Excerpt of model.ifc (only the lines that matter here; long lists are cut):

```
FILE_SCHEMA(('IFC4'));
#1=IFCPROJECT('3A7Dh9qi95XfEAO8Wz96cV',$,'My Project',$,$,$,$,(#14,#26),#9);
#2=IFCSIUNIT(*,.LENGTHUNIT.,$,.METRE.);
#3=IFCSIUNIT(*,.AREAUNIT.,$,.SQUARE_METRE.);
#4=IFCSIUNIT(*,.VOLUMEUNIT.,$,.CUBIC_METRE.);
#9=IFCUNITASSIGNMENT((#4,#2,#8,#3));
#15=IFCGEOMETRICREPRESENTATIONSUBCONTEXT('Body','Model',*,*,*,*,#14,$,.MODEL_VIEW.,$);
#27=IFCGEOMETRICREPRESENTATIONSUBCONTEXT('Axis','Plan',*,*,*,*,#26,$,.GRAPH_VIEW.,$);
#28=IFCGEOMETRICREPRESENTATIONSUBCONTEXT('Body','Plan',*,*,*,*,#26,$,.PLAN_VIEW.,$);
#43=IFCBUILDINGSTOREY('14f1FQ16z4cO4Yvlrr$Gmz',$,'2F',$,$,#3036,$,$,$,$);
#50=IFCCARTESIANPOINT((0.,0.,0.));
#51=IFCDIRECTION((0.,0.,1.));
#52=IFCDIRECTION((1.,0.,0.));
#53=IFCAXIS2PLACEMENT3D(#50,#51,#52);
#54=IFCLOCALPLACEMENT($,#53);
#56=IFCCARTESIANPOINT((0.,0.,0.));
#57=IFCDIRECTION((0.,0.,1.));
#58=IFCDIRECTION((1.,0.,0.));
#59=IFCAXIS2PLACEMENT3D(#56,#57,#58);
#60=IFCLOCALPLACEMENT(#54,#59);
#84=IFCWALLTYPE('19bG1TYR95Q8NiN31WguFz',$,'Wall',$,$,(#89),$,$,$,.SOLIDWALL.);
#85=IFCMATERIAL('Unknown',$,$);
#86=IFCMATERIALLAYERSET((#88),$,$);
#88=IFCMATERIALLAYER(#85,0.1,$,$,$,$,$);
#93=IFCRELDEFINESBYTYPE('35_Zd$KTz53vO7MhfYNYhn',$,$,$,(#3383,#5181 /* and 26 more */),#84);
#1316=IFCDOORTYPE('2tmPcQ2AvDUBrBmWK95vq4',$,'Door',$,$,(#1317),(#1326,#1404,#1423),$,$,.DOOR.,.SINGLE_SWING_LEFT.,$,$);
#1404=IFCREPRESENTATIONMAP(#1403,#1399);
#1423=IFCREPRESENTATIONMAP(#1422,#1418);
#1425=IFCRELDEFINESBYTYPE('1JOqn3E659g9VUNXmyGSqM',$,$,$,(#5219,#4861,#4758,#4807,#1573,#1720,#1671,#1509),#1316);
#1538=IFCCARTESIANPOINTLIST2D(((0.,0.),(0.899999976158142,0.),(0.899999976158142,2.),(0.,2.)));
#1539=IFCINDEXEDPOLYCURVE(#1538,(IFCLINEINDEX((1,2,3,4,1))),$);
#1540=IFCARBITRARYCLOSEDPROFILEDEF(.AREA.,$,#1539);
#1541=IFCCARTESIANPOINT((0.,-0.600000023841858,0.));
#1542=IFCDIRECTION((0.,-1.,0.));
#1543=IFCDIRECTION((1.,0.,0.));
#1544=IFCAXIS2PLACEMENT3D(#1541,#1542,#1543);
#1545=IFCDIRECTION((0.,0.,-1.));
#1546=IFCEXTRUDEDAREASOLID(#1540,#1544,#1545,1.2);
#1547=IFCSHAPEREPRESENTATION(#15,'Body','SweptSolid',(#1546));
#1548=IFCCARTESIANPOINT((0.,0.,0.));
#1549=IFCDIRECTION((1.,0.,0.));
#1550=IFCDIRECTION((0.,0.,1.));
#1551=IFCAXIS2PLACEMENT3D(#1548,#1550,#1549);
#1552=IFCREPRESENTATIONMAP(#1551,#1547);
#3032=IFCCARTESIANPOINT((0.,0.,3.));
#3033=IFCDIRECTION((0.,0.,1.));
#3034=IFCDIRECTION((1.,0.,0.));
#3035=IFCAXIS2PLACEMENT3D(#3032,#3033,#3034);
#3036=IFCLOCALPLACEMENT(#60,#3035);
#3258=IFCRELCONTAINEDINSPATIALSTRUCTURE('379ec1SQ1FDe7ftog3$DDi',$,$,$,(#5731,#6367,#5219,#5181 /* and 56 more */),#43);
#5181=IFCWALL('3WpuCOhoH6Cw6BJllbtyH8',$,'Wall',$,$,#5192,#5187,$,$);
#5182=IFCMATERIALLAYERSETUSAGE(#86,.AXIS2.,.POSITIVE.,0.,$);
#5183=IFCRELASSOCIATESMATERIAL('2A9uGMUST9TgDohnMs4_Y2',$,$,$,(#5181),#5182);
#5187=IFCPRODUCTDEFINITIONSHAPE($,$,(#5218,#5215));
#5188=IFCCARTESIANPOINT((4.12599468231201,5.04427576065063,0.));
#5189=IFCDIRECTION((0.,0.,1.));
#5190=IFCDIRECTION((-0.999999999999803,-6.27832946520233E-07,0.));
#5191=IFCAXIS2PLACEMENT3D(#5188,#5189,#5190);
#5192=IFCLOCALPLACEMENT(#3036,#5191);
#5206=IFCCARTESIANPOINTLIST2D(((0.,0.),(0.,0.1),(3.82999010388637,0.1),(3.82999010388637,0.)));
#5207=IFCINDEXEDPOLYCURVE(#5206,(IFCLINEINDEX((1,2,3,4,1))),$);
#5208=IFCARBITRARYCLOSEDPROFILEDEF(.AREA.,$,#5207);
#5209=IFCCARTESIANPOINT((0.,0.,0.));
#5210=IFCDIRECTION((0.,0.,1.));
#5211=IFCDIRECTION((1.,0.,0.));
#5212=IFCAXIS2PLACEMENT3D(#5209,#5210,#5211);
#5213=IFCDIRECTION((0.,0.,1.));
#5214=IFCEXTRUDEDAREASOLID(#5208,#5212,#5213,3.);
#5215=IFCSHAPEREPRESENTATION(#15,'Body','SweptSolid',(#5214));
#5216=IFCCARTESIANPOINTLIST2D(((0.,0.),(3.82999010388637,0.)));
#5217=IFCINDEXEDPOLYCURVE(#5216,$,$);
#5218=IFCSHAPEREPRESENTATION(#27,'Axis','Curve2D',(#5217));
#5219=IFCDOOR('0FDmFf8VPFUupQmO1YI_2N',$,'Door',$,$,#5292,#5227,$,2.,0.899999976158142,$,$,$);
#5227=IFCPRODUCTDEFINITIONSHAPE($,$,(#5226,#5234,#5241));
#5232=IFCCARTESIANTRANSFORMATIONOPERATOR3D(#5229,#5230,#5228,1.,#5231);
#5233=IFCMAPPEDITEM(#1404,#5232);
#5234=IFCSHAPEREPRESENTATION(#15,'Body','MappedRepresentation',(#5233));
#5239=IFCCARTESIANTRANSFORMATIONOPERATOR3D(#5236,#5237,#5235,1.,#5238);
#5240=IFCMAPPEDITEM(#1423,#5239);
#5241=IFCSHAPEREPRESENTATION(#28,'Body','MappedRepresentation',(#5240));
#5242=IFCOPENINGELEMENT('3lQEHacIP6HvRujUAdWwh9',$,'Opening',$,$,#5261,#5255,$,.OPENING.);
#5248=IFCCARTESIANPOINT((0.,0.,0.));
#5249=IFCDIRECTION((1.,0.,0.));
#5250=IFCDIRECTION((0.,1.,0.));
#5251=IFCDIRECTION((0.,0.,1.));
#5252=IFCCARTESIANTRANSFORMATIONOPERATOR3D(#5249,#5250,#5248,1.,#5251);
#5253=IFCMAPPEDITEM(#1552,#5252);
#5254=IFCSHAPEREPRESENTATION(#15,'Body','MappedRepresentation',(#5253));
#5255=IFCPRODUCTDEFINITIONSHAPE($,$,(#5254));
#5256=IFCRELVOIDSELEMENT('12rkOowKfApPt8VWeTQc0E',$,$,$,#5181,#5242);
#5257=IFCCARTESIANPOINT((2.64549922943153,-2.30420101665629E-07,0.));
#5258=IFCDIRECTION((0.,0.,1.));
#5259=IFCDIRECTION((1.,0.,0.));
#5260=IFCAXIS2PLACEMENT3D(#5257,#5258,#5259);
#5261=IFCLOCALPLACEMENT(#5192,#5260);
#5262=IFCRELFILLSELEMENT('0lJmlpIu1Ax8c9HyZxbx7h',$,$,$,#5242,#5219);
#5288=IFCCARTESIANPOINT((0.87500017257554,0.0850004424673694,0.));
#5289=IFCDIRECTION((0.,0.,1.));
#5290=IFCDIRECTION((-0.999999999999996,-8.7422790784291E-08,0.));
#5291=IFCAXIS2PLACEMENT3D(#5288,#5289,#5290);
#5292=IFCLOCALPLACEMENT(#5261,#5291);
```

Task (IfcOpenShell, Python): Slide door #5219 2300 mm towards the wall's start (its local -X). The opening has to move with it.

```python
import ifcopenshell
import ifcopenshell.api.geometry
import ifcopenshell.util.placement
import ifcopenshell.util.unit

model = ifcopenshell.open("model.ifc")
unit_scale = ifcopenshell.util.unit.calculate_unit_scale(model)

door = model.by_id(5219)
opening = door.FillsVoids[0].RelatingOpeningElement
wall = opening.VoidsElements[0].RelatingBuildingElement

wall_matrix = ifcopenshell.util.placement.get_local_placement(wall.ObjectPlacement)
shift = wall_matrix[:3, 0] * -2.3 / unit_scale
before = ifcopenshell.util.placement.get_local_placement(door.ObjectPlacement)[:3, 3].copy()

# The door is placed relative to its opening, so it follows when the opening moves.
matrix = ifcopenshell.util.placement.get_local_placement(opening.ObjectPlacement)
matrix[:3, 3] += shift
ifcopenshell.api.geometry.edit_object_placement(
    model, product=opening, matrix=matrix, is_si=False, should_transform_children=True
)

after = ifcopenshell.util.placement.get_local_placement(door.ObjectPlacement)[:3, 3]
print("door moved by", (after - before).round(3) + 0.0)

model.write("model-out.ifc")
```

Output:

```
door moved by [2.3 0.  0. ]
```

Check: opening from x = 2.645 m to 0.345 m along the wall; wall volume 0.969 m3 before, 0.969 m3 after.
